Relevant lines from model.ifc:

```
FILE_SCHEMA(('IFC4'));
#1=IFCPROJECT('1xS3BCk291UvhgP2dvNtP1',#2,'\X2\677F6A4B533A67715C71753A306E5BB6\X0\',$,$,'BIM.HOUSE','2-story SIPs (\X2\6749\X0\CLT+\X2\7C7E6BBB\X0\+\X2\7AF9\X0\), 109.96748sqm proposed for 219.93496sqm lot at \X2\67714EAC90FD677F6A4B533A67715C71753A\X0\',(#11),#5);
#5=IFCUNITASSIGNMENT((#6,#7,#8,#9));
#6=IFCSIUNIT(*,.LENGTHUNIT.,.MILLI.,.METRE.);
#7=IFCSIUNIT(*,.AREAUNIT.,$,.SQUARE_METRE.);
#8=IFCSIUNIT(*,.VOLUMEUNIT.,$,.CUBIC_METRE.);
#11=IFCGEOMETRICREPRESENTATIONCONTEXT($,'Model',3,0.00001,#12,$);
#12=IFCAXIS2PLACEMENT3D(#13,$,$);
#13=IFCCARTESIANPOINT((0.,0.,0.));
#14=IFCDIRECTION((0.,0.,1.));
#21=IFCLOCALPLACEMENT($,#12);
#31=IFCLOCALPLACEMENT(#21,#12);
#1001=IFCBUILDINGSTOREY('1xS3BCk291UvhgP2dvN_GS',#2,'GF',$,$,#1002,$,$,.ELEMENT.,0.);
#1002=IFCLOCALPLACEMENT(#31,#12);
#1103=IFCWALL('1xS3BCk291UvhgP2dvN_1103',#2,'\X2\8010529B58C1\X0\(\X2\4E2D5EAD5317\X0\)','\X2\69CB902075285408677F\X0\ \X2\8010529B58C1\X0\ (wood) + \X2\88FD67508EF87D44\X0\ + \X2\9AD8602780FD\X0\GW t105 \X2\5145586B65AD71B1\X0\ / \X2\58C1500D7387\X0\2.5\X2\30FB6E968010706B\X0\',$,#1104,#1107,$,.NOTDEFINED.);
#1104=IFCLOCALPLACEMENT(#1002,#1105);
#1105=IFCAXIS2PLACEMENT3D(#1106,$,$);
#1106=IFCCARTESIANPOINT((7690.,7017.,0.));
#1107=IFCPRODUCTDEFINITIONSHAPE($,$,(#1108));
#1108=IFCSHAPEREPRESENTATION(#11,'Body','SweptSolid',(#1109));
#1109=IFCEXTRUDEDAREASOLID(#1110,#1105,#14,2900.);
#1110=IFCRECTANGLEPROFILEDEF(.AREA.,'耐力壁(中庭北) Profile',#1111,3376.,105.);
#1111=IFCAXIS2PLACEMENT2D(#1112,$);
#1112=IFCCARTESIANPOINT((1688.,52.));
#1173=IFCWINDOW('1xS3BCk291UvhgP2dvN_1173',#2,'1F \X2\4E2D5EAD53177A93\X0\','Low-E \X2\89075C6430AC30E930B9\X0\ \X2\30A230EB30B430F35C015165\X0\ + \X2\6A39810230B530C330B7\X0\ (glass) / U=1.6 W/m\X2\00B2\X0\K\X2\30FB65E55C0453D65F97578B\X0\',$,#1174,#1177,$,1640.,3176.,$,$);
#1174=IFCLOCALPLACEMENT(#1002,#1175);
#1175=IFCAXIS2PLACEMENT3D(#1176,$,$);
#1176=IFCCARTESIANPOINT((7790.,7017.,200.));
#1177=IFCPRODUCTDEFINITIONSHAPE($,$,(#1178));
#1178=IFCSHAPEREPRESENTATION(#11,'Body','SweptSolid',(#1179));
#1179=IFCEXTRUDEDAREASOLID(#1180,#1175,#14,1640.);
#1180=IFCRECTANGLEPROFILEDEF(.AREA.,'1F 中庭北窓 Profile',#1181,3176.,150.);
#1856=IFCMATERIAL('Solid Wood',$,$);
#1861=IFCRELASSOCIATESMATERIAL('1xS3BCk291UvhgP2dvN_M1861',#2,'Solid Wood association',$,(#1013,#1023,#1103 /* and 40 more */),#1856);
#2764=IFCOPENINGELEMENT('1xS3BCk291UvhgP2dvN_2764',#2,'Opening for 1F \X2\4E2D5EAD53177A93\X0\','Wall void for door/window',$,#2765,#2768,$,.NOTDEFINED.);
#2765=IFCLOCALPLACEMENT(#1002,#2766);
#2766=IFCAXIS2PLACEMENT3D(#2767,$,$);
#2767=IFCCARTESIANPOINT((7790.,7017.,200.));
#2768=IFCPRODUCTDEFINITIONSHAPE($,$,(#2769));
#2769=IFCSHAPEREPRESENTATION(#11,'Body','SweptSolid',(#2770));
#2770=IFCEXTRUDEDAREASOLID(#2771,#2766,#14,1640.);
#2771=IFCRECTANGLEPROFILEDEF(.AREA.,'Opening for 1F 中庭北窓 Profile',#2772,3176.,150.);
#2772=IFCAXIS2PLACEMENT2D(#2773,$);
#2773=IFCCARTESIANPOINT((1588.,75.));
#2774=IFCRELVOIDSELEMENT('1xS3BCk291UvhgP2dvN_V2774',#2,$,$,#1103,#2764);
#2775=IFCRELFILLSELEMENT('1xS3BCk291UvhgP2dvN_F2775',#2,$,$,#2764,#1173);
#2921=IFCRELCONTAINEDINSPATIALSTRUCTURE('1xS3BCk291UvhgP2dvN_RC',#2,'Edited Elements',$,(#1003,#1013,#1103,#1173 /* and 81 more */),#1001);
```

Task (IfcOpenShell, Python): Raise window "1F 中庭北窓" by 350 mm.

```python
import numpy as np
import ifcopenshell
import ifcopenshell.api.geometry
import ifcopenshell.util.placement
import ifcopenshell.util.unit

model = ifcopenshell.open("model.ifc")
unit_scale = ifcopenshell.util.unit.calculate_unit_scale(model)

window = model.by_id(1173)
opening = window.FillsVoids[0].RelatingOpeningElement
dz = 0.35 / unit_scale

shift = np.array([0.0, 0.0, dz])
# The window is not placed relative to its opening, so move both.
for product in (opening, window):
    matrix = ifcopenshell.util.placement.get_local_placement(product.ObjectPlacement)
    matrix[:3, 3] += shift
    ifcopenshell.api.geometry.edit_object_placement(model, product=product, matrix=matrix, is_si=False)

print(f"moved by {dz * unit_scale:+.3f} m")

model.write("model_rev.ifc")
```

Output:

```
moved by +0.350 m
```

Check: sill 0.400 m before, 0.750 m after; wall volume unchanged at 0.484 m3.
